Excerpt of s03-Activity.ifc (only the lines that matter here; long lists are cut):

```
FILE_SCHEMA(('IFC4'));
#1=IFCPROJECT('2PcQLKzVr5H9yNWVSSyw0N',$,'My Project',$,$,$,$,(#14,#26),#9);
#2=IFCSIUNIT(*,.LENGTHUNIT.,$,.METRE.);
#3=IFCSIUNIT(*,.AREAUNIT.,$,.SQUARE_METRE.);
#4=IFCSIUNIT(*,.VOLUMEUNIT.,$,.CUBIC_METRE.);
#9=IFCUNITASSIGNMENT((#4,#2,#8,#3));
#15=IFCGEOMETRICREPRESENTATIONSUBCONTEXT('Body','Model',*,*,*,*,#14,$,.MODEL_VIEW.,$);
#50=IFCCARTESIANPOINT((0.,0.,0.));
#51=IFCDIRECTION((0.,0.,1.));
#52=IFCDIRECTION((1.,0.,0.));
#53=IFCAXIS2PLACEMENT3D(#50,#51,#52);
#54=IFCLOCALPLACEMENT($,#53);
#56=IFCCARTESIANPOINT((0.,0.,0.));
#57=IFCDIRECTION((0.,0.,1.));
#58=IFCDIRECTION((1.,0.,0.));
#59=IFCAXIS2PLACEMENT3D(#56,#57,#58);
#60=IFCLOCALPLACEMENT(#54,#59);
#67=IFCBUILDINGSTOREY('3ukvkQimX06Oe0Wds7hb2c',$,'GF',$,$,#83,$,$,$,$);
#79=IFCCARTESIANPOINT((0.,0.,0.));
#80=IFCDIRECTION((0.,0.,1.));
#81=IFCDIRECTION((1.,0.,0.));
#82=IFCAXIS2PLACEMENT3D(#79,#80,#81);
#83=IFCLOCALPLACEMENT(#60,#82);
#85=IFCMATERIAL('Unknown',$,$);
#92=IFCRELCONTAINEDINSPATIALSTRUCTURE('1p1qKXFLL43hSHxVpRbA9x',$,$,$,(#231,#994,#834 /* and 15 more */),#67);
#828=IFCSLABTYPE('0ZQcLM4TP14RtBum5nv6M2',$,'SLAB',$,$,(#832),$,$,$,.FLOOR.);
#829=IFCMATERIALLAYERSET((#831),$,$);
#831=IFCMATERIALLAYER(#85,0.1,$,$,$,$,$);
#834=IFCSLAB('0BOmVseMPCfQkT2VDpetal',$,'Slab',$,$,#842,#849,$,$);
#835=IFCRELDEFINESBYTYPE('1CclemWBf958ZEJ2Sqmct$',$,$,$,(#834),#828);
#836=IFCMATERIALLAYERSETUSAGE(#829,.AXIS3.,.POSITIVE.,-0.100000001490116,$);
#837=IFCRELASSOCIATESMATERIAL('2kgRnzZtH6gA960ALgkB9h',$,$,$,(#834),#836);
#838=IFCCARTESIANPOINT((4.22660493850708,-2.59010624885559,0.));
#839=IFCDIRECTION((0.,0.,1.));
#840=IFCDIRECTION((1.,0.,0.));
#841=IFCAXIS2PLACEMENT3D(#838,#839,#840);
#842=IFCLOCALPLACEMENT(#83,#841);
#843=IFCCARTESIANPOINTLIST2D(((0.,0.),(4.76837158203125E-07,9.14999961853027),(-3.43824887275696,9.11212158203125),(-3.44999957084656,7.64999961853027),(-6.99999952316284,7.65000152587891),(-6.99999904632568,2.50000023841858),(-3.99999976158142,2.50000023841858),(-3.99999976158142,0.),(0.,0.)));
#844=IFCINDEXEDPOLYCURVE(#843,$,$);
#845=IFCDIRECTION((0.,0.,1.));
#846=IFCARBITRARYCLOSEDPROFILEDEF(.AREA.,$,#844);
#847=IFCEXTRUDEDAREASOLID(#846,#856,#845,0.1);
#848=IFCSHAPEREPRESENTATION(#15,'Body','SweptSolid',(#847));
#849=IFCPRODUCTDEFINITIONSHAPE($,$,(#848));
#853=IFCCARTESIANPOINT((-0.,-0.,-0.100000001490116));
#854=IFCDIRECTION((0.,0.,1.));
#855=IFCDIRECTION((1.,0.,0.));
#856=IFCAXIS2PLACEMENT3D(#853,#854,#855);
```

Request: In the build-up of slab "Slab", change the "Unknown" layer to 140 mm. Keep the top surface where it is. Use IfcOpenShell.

```python
import ifcopenshell
import ifcopenshell.util.element
import ifcopenshell.util.representation
import ifcopenshell.util.unit

model = ifcopenshell.open("s03-Activity.ifc")
unit_scale = ifcopenshell.util.unit.calculate_unit_scale(model)

layer_set = model.by_id(829)
layer = next(l for l in layer_set.MaterialLayers if l.Material and l.Material.Name == "Unknown")
change = 0.14 / unit_scale - layer.LayerThickness
layer.LayerThickness += change

# Geometry does not follow the layer set by itself.
slabs = [e for e in ifcopenshell.util.element.get_elements_by_material(model, layer_set) if e.is_a("IfcSlab")]
for slab in sorted(slabs, key=lambda e: e.id()):
    body = ifcopenshell.util.representation.get_representation(slab, "Model", "Body")
    solid = body.Items[0]
    old_depth = solid.Depth
    solid.Depth += change
    # Extruded upwards: lower the start of the extrusion so the top stays.
    x, y, z = solid.Position.Location.Coordinates
    solid.Position.Location = model.createIfcCartesianPoint((x, y, z - change))
    print(slab.id(), f"{old_depth:g} -> {solid.Depth:g}")

# The layers are counted up from the underside, which has moved.
for usage in {ifcopenshell.util.element.get_material(slab) for slab in slabs}:
    usage.OffsetFromReferenceLine -= change

model.write("s03-Activity-out.ifc")
```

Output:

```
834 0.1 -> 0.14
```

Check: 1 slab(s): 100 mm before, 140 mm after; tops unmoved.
